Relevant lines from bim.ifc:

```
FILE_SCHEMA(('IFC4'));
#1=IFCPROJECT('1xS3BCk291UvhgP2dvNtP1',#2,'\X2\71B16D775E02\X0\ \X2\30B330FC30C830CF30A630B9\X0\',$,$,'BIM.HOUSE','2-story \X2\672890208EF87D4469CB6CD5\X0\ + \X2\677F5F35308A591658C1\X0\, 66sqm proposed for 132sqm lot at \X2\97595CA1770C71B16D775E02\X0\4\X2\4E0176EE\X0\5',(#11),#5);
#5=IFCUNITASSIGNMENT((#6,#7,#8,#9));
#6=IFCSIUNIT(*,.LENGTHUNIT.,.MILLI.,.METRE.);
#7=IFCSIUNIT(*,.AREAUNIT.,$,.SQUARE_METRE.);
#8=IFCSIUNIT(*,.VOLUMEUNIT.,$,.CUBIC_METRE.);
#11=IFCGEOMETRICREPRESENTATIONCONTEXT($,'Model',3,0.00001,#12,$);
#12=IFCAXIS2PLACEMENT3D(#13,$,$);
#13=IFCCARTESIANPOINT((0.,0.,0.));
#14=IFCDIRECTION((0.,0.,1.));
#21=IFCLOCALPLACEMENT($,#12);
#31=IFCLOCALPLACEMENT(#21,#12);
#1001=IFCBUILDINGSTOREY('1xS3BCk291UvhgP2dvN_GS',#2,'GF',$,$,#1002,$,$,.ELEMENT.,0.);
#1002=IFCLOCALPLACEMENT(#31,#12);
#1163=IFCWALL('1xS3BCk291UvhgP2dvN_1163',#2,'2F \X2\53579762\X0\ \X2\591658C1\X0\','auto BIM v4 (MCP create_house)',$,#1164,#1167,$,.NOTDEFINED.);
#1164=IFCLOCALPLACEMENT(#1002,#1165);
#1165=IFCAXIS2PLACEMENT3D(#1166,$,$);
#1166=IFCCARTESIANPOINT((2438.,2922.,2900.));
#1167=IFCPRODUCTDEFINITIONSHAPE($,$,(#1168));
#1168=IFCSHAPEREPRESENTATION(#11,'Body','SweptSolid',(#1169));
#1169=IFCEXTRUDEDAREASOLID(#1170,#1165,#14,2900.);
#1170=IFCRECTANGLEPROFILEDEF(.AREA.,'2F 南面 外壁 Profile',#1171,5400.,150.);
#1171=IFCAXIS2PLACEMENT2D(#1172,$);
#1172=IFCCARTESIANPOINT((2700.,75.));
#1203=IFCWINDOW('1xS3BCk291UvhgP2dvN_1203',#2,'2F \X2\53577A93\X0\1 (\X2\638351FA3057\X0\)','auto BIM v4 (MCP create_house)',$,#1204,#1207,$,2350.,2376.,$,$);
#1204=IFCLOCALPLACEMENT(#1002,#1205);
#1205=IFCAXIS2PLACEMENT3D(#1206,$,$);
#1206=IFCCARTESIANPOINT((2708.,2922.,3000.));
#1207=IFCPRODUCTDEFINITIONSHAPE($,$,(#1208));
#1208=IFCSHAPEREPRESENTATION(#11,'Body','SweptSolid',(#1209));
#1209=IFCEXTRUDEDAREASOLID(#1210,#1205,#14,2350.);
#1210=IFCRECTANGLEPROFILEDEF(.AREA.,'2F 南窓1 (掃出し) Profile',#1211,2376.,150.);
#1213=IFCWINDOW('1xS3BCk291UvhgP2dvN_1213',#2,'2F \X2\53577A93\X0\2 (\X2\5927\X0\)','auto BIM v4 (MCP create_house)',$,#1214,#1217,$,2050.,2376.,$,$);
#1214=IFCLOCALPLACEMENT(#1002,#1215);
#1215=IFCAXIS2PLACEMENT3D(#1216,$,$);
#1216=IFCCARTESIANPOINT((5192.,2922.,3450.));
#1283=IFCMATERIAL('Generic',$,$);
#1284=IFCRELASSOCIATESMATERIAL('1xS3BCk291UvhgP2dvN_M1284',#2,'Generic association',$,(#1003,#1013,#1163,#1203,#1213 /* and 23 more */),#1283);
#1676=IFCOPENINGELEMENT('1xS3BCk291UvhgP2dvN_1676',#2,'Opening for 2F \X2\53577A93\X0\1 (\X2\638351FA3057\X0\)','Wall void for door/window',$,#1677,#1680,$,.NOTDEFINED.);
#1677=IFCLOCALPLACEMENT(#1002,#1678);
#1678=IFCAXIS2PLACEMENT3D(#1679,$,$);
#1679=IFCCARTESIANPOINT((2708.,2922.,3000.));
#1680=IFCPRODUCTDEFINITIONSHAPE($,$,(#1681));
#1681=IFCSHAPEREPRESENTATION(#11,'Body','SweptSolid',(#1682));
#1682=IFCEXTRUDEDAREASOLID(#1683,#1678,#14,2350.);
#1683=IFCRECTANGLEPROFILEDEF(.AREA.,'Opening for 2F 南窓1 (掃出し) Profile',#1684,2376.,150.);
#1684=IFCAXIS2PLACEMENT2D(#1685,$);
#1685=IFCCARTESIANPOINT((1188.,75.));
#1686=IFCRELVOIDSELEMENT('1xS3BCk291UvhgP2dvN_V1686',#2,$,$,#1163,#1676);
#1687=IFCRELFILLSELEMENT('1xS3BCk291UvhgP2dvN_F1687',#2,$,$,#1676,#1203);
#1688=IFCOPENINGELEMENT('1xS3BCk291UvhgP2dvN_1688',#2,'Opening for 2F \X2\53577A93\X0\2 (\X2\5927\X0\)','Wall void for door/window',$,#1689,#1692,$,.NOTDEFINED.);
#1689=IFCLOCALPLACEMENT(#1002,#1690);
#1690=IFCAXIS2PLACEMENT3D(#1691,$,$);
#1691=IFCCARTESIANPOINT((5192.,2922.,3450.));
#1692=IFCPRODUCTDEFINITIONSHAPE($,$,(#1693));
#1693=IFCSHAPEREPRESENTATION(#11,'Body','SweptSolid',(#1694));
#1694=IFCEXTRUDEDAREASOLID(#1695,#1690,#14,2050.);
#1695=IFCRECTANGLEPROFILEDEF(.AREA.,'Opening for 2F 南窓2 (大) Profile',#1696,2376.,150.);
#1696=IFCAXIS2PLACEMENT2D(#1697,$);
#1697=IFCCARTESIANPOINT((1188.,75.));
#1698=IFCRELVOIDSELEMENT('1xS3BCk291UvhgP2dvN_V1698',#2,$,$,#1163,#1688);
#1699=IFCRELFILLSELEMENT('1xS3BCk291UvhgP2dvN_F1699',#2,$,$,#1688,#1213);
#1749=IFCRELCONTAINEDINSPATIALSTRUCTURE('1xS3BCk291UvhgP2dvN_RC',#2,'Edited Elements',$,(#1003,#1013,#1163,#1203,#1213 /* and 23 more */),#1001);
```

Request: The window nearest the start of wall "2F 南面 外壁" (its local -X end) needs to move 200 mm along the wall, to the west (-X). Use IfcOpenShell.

```python
import ifcopenshell
import ifcopenshell.api.geometry
import ifcopenshell.util.placement

model = ifcopenshell.open("bim.ifc")

window = model.by_guid("1xS3BCk291UvhgP2dvN_1203")
opening = window.FillsVoids[0].RelatingOpeningElement
wall = opening.VoidsElements[0].RelatingBuildingElement

wall_matrix = ifcopenshell.util.placement.get_local_placement(wall.ObjectPlacement)
shift = wall_matrix[:3, 0] * -200.0
before = ifcopenshell.util.placement.get_local_placement(window.ObjectPlacement)[:3, 3].copy()

# The window is not placed relative to its opening, so move both.
for product in (opening, window):
    matrix = ifcopenshell.util.placement.get_local_placement(product.ObjectPlacement)
    matrix[:3, 3] += shift
    ifcopenshell.api.geometry.edit_object_placement(model, product=product, matrix=matrix, is_si=False)

after = ifcopenshell.util.placement.get_local_placement(window.ObjectPlacement)[:3, 3]
print("window moved by", (after - before).round(3) + 0.0)

model.write("bim_updated.ifc")
```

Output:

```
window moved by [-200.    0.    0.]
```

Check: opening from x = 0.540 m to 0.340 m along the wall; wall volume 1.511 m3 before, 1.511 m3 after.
